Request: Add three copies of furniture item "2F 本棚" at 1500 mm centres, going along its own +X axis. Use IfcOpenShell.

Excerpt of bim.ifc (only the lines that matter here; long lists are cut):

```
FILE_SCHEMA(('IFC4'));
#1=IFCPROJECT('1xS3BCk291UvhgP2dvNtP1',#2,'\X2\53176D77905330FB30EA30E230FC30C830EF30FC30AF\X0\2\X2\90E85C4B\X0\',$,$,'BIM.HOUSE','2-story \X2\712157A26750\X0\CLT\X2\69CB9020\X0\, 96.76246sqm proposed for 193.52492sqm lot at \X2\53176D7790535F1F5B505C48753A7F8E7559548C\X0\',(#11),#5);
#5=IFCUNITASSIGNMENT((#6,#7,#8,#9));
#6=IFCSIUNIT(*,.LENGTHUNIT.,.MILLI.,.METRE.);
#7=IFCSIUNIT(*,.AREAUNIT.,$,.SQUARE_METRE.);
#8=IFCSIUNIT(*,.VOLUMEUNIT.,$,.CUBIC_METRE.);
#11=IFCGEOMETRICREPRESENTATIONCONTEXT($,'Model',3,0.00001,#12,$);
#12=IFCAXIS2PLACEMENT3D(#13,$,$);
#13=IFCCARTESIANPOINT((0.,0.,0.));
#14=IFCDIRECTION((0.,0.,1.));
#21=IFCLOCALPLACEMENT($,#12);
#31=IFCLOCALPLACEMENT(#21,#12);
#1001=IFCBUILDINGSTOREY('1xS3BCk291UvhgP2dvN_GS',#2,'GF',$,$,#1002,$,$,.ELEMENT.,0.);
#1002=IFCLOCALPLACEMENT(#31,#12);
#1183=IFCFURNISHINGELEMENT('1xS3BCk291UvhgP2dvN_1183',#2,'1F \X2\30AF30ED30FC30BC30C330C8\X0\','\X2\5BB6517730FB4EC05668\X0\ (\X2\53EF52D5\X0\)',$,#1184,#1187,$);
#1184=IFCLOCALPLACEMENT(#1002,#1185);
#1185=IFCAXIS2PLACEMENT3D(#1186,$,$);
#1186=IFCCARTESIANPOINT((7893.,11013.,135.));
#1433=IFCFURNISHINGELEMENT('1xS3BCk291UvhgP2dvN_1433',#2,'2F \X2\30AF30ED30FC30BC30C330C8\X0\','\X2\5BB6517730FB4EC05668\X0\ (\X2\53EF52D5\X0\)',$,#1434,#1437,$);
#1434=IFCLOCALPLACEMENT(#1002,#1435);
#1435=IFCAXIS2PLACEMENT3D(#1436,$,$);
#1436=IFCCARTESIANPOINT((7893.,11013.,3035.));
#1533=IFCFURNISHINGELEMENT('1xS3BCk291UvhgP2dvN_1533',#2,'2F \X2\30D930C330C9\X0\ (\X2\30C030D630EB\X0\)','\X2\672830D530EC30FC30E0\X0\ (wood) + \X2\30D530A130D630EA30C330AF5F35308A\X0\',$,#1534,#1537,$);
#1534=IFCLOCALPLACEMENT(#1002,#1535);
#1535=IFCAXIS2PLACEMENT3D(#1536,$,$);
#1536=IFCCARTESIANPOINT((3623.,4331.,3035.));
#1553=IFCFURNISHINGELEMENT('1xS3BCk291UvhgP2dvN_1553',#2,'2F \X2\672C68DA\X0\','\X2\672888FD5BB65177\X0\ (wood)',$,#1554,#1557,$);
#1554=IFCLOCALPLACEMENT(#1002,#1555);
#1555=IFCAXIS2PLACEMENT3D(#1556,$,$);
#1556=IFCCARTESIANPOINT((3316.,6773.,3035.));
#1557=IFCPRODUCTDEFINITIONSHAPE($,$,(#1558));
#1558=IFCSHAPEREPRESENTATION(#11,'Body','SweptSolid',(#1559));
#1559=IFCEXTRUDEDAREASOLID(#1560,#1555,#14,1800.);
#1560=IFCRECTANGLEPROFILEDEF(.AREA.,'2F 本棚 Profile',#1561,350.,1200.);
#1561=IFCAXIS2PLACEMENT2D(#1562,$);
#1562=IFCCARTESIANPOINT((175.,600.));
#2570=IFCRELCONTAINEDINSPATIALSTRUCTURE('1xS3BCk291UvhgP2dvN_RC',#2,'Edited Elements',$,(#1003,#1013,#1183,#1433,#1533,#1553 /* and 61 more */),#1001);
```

```python
import ifcopenshell
import ifcopenshell.api.geometry
import ifcopenshell.api.root
import ifcopenshell.util.element
import ifcopenshell.util.placement

model = ifcopenshell.open("bim.ifc")


def reuse_history(source, copy):
    """copy_class also copies each property set's owner history, people and application; keep the originals."""
    for rel in copy.IsDefinedBy:
        if rel.is_a("IfcRelDefinesByProperties") and (history := rel.RelatingPropertyDefinition.OwnerHistory):
            rel.RelatingPropertyDefinition.OwnerHistory = source.OwnerHistory
            ifcopenshell.util.element.remove_deep2(model, history)


source = model.by_guid("1xS3BCk291UvhgP2dvN_1553")
base = ifcopenshell.util.placement.get_local_placement(source.ObjectPlacement)
step = base[:3, 0] * 1500.0

for i in range(1, 4):
    copy = ifcopenshell.api.root.copy_class(model, product=source)
    copy.Representation = ifcopenshell.util.element.copy_deep(
        model, source.Representation, exclude=["IfcGeometricRepresentationContext", "IfcRepresentationMap"]
    )
    reuse_history(source, copy)
    matrix = base.copy()
    matrix[:3, 3] += i * step
    print("added at", matrix[:3, 3].round(3) + 0.0)
    ifcopenshell.api.geometry.edit_object_placement(model, product=copy, matrix=matrix, is_si=False)

model.write("bim_updated.ifc")
```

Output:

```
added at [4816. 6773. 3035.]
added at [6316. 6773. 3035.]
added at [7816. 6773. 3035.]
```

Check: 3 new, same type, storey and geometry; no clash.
